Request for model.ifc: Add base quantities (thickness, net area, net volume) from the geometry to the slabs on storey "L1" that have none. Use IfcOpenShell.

First a look at what the model holds.

```python
import ifcopenshell
import ifcopenshell.util.element
import ifcopenshell.util.unit

model = ifcopenshell.open("model.ifc")
print(model.schema)
for unit_type in ("LENGTHUNIT", "AREAUNIT", "VOLUMEUNIT"):
    print(unit_type, ifcopenshell.util.unit.calculate_unit_scale(model, unit_type))
storey = next(s for s in model.by_type("IfcBuildingStorey") if s.Name == "L1")
slabs = [e for e in ifcopenshell.util.element.get_decomposition(storey) if e.is_a("IfcSlab")]
for e in sorted(slabs, key=lambda e: e.id()):
    print(e.id(), e.is_a(), e.Name, list(ifcopenshell.util.element.get_psets(e, qtos_only=True)), sep=" | ")
```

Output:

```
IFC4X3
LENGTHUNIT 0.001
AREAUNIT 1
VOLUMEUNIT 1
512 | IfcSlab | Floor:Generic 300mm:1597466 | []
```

```python
import ifcopenshell
import ifcopenshell.api.pset
import ifcopenshell.geom
import ifcopenshell.util.element
import ifcopenshell.util.shape
import ifcopenshell.util.unit

model = ifcopenshell.open("model.ifc")
unit_scale = ifcopenshell.util.unit.calculate_unit_scale(model)
area_scale = ifcopenshell.util.unit.calculate_unit_scale(model, "AREAUNIT")
volume_scale = ifcopenshell.util.unit.calculate_unit_scale(model, "VOLUMEUNIT")
settings = ifcopenshell.geom.settings()

storey = next(s for s in model.by_type("IfcBuildingStorey") if s.Name == "L1")
slabs = [e for e in ifcopenshell.util.element.get_decomposition(storey) if e.is_a("IfcSlab")]

for e in sorted(slabs, key=lambda e: e.id()):
    if ifcopenshell.util.element.get_psets(e, qtos_only=True, should_inherit=False):
        continue
    # Geometry comes back in metres, in the element's own axes.
    shape = ifcopenshell.geom.create_shape(settings, e)
    values = {
        "Width": ifcopenshell.util.shape.get_z(shape.geometry) / unit_scale,
        "NetArea": ifcopenshell.util.shape.get_footprint_area(shape.geometry) / area_scale,
        "NetVolume": ifcopenshell.util.shape.get_volume(shape.geometry) / volume_scale,
    }
    qto = ifcopenshell.api.pset.add_qto(model, product=e, name="Qto_SlabBaseQuantities")
    ifcopenshell.api.pset.edit_qto(model, qto=qto, properties=values)
    print(e.id(), {k: round(v, 3) for k, v in values.items()})

model.write("model-out.ifc")
```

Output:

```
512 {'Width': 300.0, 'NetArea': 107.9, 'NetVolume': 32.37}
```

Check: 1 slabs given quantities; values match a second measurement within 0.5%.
